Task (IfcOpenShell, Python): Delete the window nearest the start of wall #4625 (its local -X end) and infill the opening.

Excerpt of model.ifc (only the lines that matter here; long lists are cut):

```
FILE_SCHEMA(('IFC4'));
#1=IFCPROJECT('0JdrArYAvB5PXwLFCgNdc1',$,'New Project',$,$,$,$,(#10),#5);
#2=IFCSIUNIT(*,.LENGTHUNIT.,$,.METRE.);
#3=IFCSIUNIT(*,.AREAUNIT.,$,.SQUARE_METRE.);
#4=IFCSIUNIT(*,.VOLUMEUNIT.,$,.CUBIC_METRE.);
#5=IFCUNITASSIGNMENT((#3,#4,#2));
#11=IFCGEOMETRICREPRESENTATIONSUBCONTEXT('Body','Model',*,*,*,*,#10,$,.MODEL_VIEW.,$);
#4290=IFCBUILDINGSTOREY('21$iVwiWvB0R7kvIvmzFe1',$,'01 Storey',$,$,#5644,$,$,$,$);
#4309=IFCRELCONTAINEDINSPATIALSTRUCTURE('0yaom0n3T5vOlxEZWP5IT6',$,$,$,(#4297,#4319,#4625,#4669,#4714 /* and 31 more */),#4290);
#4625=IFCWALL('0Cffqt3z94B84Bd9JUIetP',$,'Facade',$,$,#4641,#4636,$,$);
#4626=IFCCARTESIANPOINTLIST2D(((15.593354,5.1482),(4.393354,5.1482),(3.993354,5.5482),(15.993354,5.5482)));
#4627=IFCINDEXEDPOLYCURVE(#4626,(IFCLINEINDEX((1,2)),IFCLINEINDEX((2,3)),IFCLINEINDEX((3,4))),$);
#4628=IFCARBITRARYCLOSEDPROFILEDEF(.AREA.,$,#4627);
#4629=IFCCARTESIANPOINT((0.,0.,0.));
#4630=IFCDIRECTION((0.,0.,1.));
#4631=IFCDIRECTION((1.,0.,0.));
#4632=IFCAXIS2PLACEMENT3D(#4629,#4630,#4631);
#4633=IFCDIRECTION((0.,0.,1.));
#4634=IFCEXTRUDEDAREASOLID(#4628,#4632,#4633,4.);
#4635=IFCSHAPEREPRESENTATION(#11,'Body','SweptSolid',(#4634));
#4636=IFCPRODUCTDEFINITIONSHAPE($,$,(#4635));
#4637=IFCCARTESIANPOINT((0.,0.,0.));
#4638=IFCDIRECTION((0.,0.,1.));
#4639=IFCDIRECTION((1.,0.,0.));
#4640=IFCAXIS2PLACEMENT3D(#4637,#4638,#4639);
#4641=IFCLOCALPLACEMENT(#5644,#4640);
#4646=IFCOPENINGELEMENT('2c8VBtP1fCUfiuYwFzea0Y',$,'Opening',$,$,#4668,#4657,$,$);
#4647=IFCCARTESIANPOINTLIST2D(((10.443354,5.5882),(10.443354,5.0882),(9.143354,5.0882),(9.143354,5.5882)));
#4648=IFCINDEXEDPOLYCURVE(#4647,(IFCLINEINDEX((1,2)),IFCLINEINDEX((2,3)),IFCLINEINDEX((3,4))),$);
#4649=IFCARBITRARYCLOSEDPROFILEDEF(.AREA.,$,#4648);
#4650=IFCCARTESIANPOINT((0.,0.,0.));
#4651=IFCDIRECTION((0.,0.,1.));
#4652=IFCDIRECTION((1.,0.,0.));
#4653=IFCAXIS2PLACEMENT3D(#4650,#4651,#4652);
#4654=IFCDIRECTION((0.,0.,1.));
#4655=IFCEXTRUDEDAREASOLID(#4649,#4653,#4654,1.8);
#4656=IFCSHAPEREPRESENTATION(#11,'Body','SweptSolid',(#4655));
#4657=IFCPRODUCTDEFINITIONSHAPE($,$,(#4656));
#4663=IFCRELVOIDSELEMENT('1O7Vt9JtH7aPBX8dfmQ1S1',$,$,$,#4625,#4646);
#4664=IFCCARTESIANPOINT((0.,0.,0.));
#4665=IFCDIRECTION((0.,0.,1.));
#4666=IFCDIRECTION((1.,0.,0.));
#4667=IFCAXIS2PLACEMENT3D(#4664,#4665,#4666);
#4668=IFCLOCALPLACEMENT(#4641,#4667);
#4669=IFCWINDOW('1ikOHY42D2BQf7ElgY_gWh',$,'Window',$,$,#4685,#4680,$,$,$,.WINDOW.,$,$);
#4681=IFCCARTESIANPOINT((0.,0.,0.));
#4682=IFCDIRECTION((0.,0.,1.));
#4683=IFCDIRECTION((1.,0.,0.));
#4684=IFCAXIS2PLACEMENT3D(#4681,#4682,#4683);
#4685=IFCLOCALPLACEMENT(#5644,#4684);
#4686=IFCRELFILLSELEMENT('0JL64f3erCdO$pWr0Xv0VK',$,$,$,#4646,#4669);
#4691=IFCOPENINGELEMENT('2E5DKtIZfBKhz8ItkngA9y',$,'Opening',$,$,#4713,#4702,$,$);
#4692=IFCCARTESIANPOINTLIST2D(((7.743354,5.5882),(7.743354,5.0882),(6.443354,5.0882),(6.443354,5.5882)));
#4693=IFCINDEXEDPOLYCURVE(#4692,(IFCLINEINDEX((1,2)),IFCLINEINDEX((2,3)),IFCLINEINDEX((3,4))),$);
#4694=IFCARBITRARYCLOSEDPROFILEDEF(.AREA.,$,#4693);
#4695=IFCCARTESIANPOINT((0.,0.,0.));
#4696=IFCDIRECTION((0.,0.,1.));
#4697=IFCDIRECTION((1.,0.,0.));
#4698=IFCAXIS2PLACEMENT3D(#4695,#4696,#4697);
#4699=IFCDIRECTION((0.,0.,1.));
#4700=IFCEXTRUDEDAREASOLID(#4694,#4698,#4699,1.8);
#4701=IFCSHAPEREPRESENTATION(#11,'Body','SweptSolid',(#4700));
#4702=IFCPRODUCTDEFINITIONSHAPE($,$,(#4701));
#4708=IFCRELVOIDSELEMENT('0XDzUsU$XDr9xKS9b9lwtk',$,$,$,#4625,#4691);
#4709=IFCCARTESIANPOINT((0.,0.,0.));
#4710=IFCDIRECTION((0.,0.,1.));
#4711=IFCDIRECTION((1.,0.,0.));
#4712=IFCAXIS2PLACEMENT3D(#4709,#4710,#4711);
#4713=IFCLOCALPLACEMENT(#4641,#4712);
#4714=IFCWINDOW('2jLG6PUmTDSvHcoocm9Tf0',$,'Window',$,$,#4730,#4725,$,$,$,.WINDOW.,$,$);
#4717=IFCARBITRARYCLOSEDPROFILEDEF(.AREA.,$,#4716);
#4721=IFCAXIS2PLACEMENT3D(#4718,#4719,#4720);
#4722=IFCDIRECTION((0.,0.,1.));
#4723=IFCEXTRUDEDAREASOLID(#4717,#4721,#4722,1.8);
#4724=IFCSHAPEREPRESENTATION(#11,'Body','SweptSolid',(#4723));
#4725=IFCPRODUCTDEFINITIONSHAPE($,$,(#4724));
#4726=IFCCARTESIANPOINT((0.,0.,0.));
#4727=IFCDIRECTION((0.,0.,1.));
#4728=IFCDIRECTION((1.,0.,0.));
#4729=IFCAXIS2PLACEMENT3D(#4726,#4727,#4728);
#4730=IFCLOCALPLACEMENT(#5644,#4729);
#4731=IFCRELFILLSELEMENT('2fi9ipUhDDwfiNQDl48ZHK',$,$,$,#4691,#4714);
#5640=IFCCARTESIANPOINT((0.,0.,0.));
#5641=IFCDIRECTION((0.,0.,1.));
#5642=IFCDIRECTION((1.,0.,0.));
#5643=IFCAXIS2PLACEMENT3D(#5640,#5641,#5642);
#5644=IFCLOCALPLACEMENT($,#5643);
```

```python
import ifcopenshell
import ifcopenshell.api.feature
import ifcopenshell.api.root
import ifcopenshell.geom
import ifcopenshell.util.shape

model = ifcopenshell.open("model.ifc")
settings = ifcopenshell.geom.settings()


def volume(element):
    """Net volume in cubic metres, openings subtracted."""
    shape = ifcopenshell.geom.create_shape(settings, element)
    return ifcopenshell.util.shape.get_volume(shape.geometry)


window = model.by_guid("2jLG6PUmTDSvHcoocm9Tf0")
opening = window.FillsVoids[0].RelatingOpeningElement
wall = opening.VoidsElements[0].RelatingBuildingElement
before = volume(wall)

ifcopenshell.api.root.remove_product(model, product=window)
ifcopenshell.api.feature.remove_feature(model, feature=opening)

after = volume(wall)

print(f"wall volume {before:.3f} -> {after:.3f} m3")

model.write("model_updated.ifc")
```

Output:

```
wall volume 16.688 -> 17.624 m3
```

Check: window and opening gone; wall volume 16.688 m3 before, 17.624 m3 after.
